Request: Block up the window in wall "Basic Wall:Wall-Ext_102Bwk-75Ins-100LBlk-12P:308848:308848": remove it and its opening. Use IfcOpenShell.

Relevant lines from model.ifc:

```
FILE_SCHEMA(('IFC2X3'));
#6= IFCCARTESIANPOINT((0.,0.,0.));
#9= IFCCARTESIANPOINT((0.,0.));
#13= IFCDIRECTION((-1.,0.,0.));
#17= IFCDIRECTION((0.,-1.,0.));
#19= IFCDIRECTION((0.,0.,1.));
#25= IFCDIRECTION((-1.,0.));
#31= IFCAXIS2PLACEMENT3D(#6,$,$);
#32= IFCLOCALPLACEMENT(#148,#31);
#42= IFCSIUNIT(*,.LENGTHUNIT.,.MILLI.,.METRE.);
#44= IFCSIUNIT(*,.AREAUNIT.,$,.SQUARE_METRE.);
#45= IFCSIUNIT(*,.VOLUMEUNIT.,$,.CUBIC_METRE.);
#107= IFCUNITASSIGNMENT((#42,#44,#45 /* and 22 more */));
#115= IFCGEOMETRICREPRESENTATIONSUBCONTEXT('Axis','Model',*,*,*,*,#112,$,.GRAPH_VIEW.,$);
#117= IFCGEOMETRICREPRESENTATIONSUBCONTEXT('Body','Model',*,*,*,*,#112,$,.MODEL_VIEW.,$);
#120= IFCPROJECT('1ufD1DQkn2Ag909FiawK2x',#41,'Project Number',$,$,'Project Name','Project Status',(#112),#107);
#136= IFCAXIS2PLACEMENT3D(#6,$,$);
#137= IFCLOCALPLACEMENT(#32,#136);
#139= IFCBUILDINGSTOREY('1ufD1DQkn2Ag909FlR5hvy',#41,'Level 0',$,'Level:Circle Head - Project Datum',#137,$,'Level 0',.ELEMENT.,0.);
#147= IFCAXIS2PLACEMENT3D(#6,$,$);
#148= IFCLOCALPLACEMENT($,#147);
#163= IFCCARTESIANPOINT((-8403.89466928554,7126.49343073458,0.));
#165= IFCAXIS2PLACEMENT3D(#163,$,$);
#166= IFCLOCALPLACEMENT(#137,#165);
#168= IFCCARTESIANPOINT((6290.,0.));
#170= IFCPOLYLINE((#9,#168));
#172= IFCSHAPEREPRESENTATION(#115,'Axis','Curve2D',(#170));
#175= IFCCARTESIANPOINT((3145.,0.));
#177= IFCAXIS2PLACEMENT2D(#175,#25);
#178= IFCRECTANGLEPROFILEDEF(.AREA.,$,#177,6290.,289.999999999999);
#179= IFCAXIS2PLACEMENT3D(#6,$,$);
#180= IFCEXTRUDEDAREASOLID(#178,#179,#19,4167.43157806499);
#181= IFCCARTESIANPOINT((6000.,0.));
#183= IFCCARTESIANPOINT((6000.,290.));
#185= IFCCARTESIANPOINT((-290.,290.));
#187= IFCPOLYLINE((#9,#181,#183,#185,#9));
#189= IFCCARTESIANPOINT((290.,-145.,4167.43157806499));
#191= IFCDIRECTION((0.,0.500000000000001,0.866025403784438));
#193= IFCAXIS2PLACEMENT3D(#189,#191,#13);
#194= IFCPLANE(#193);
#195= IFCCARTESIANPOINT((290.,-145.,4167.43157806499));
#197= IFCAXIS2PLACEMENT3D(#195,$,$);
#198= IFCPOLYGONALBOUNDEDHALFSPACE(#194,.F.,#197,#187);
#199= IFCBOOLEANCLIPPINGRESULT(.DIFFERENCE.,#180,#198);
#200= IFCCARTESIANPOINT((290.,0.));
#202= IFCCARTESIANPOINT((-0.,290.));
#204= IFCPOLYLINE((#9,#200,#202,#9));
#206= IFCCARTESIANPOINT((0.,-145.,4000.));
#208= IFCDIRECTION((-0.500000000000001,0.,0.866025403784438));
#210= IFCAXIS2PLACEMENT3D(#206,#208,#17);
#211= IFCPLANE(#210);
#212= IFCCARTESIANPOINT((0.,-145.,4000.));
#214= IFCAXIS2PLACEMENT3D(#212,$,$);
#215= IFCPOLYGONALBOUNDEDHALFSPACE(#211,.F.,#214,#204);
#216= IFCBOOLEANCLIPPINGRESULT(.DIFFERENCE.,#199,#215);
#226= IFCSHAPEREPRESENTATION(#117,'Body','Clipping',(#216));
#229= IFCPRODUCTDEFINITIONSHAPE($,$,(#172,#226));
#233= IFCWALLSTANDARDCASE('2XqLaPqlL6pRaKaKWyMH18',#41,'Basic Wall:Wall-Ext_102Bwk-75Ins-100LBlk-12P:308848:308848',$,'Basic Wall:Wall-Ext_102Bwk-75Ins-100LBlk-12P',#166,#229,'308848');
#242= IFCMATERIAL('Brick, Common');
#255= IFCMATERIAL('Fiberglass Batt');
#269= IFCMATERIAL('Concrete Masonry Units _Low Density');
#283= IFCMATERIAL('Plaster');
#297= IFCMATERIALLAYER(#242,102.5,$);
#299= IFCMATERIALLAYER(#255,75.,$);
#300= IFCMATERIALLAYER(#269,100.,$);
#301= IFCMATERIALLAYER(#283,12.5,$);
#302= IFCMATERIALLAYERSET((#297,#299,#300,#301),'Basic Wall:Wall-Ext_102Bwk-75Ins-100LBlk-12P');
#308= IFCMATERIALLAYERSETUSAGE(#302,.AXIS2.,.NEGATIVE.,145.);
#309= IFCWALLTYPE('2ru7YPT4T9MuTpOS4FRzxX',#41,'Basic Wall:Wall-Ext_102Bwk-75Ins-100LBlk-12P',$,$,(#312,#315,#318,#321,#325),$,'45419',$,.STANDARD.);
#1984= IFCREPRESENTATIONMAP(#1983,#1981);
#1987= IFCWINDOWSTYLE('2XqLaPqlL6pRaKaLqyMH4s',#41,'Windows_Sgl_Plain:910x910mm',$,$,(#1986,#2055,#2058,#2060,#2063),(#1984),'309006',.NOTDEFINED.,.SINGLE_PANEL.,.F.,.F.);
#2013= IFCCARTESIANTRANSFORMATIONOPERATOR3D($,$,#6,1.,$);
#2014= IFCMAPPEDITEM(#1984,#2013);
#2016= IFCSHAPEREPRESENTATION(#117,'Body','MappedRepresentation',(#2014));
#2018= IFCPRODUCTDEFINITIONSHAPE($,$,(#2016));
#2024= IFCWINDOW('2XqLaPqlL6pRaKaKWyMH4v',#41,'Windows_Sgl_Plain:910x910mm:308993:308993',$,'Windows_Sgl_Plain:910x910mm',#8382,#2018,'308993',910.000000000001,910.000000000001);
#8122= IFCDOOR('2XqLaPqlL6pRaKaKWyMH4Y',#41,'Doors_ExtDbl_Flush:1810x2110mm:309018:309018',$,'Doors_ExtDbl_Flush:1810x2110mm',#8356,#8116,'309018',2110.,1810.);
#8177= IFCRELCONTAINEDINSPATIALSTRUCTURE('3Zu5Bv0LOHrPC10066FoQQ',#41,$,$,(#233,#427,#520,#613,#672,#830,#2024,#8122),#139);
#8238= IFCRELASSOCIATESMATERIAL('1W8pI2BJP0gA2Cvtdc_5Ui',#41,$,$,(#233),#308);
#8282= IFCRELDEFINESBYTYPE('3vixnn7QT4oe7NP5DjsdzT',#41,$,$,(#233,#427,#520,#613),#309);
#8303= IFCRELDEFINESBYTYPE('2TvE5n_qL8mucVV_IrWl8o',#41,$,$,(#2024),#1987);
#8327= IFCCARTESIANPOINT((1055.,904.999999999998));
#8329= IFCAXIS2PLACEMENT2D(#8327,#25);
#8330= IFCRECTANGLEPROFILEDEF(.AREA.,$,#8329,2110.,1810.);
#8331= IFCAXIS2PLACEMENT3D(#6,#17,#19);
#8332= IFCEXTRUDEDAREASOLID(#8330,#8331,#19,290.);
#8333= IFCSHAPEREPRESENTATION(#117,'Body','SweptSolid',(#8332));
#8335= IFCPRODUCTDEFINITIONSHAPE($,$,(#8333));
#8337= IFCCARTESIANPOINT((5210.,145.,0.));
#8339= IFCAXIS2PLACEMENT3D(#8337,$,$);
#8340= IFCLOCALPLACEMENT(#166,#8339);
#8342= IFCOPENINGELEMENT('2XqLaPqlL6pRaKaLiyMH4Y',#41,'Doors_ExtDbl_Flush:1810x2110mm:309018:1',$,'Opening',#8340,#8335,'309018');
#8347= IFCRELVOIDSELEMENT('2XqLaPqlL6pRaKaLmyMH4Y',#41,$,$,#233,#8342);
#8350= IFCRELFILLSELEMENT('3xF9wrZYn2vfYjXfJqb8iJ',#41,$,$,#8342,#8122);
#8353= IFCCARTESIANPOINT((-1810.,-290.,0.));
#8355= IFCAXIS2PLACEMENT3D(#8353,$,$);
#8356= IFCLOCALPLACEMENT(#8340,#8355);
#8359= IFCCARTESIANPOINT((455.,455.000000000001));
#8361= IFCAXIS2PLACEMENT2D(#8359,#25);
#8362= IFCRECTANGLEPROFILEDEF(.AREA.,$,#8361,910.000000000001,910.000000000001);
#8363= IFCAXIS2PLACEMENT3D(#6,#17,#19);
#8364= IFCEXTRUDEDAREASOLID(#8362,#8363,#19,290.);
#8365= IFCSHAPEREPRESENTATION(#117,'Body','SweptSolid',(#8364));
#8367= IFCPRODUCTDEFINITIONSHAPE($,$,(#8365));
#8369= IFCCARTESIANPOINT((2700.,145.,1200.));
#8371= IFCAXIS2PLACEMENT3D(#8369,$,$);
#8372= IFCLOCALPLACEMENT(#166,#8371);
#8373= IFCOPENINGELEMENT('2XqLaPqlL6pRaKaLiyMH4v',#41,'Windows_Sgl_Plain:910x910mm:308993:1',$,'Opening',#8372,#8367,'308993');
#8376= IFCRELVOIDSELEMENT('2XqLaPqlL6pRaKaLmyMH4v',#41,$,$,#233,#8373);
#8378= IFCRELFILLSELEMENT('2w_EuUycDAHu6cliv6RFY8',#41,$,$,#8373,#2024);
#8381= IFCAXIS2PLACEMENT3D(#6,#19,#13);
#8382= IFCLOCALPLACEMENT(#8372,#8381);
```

```python
import ifcopenshell
import ifcopenshell.api.feature
import ifcopenshell.api.root
import ifcopenshell.geom
import ifcopenshell.util.shape

model = ifcopenshell.open("model.ifc")
settings = ifcopenshell.geom.settings()


def volume(element):
    """Net volume in cubic metres, openings subtracted."""
    shape = ifcopenshell.geom.create_shape(settings, element)
    return ifcopenshell.util.shape.get_volume(shape.geometry)


window = model.by_id(2024)
opening = window.FillsVoids[0].RelatingOpeningElement
wall = opening.VoidsElements[0].RelatingBuildingElement
before = volume(wall)

ifcopenshell.api.root.remove_product(model, product=window)
ifcopenshell.api.feature.remove_feature(model, feature=opening)

after = volume(wall)

print(f"wall volume {before:.3f} -> {after:.3f} m3")

model.write("model-out.ifc")
```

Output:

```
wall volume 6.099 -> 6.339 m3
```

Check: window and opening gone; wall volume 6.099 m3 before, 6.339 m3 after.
